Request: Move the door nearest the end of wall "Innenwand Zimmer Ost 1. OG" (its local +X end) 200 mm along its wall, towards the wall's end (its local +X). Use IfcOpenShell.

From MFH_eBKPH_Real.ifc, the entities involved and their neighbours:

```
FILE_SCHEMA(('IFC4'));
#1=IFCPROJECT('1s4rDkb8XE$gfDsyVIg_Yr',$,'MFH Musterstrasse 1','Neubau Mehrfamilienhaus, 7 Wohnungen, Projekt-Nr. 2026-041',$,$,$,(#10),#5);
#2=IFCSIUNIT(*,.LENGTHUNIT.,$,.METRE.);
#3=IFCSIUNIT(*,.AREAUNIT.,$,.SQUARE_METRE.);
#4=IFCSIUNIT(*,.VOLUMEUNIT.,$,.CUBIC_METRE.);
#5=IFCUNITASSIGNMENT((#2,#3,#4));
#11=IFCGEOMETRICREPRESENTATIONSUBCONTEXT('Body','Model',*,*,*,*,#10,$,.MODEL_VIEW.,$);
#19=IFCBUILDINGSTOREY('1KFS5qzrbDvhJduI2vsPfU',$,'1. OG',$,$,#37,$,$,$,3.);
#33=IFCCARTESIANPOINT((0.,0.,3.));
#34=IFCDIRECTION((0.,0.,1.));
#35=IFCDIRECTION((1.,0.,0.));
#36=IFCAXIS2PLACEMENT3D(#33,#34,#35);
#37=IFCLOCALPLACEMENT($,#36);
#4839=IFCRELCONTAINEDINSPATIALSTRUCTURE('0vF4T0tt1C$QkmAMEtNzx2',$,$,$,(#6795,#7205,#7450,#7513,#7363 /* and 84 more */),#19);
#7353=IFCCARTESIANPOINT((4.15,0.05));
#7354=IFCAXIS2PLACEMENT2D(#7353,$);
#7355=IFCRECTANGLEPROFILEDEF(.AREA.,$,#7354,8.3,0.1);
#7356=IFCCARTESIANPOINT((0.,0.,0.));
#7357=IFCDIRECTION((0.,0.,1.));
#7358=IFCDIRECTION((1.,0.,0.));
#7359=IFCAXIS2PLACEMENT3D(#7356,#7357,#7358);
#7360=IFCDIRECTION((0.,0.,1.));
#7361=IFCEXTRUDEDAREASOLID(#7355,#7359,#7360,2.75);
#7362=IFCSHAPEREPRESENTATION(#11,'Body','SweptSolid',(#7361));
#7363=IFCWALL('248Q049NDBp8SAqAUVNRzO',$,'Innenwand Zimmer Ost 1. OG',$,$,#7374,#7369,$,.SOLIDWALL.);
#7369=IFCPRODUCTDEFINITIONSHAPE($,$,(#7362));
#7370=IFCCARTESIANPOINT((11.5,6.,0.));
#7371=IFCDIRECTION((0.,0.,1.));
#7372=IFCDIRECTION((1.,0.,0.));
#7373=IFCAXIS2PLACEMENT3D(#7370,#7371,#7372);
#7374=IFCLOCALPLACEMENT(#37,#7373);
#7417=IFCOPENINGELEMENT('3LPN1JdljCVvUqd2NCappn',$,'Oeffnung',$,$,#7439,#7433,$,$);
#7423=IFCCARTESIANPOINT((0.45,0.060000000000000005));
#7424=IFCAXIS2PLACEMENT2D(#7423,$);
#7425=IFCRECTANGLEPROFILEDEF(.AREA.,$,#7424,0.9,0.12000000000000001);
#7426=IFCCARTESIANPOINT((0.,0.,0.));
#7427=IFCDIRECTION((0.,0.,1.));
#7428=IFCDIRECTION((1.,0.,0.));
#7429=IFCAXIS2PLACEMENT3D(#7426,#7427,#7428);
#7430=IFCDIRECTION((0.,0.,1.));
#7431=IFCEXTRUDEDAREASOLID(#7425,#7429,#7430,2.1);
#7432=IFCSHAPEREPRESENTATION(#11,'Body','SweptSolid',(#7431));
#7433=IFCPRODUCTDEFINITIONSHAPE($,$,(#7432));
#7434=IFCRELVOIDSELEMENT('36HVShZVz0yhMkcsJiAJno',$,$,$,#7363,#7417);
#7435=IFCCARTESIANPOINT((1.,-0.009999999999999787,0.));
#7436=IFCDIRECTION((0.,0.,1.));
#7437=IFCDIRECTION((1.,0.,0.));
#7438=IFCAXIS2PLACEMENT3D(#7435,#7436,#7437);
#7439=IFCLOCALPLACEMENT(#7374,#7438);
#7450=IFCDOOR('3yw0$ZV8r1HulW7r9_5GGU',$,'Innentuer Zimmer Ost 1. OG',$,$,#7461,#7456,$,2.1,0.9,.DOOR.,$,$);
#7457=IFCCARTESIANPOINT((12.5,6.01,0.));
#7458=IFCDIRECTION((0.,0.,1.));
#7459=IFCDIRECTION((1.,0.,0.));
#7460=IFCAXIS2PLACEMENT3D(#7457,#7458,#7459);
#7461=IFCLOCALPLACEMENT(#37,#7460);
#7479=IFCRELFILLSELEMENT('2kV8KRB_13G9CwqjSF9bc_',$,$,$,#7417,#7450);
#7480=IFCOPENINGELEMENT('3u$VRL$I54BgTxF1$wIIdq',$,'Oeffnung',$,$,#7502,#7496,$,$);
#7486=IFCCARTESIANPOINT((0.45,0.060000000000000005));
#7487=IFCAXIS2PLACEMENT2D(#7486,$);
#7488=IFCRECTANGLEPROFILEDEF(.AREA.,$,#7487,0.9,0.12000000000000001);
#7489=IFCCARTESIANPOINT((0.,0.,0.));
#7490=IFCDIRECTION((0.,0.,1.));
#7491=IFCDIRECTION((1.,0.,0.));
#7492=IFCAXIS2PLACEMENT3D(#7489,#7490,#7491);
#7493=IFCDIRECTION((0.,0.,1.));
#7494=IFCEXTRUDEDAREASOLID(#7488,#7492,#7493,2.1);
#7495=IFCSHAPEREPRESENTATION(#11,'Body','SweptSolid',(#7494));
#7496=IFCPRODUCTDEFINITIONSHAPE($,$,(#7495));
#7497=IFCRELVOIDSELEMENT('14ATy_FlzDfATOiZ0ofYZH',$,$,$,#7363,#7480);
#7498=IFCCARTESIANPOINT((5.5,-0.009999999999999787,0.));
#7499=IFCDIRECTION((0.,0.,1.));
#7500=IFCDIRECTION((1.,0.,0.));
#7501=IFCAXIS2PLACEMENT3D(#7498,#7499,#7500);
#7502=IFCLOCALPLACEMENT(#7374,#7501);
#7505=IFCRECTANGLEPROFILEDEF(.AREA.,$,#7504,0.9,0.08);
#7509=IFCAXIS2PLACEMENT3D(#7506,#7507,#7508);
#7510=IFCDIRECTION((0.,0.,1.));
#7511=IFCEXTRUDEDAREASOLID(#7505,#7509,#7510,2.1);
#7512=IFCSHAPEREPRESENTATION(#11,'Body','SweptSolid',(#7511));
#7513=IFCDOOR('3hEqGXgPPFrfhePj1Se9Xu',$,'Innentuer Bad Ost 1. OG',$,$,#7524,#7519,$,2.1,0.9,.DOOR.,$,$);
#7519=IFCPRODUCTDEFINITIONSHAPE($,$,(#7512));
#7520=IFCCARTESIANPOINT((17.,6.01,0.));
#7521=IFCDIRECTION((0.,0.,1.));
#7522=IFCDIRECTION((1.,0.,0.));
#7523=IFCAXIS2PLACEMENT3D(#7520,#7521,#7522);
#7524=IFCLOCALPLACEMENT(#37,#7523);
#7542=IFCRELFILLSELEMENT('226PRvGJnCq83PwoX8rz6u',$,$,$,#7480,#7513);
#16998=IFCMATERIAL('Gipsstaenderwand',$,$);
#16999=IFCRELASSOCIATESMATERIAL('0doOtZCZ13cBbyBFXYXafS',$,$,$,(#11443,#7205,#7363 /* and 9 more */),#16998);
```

```python
import ifcopenshell
import ifcopenshell.api.geometry
import ifcopenshell.util.placement
import ifcopenshell.util.unit

model = ifcopenshell.open("MFH_eBKPH_Real.ifc")
unit_scale = ifcopenshell.util.unit.calculate_unit_scale(model)

door = model.by_id(7513)
opening = door.FillsVoids[0].RelatingOpeningElement
wall = opening.VoidsElements[0].RelatingBuildingElement

wall_matrix = ifcopenshell.util.placement.get_local_placement(wall.ObjectPlacement)
shift = wall_matrix[:3, 0] * 0.2 / unit_scale
before = ifcopenshell.util.placement.get_local_placement(door.ObjectPlacement)[:3, 3].copy()

# The door is not placed relative to its opening, so move both.
for product in (opening, door):
    matrix = ifcopenshell.util.placement.get_local_placement(product.ObjectPlacement)
    matrix[:3, 3] += shift
    ifcopenshell.api.geometry.edit_object_placement(model, product=product, matrix=matrix, is_si=False)

after = ifcopenshell.util.placement.get_local_placement(door.ObjectPlacement)[:3, 3]
print("door moved by", (after - before).round(3) + 0.0)

model.write("MFH_eBKPH_Real_rev.ifc")
```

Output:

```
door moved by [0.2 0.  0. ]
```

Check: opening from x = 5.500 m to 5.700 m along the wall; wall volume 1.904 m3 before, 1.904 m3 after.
